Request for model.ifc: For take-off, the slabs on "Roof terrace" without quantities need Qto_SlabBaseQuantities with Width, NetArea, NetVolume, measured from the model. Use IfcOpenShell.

First a look at what the model holds.

```python
import ifcopenshell
import ifcopenshell.util.element
import ifcopenshell.util.unit

model = ifcopenshell.open("model.ifc")
print(model.schema)
for unit_type in ("LENGTHUNIT", "AREAUNIT", "VOLUMEUNIT"):
    print(unit_type, ifcopenshell.util.unit.calculate_unit_scale(model, unit_type))
storey = next(s for s in model.by_type("IfcBuildingStorey") if s.Name == "Roof terrace")
slabs = [e for e in ifcopenshell.util.element.get_decomposition(storey) if e.is_a("IfcSlab")]
for e in sorted(slabs, key=lambda e: e.id()):
    print(e.id(), e.is_a(), e.Name, list(ifcopenshell.util.element.get_psets(e, qtos_only=True)), sep=" | ")
```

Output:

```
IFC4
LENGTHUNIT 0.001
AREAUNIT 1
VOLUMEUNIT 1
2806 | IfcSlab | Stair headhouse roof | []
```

```python
import ifcopenshell
import ifcopenshell.api.pset
import ifcopenshell.geom
import ifcopenshell.util.element
import ifcopenshell.util.shape
import ifcopenshell.util.unit

model = ifcopenshell.open("model.ifc")
unit_scale = ifcopenshell.util.unit.calculate_unit_scale(model)
area_scale = ifcopenshell.util.unit.calculate_unit_scale(model, "AREAUNIT")
volume_scale = ifcopenshell.util.unit.calculate_unit_scale(model, "VOLUMEUNIT")
settings = ifcopenshell.geom.settings()

storey = next(s for s in model.by_type("IfcBuildingStorey") if s.Name == "Roof terrace")
slabs = [e for e in ifcopenshell.util.element.get_decomposition(storey) if e.is_a("IfcSlab")]

for e in sorted(slabs, key=lambda e: e.id()):
    if ifcopenshell.util.element.get_psets(e, qtos_only=True, should_inherit=False):
        continue
    # Geometry comes back in metres, in the element's own axes.
    shape = ifcopenshell.geom.create_shape(settings, e)
    values = {
        "Width": ifcopenshell.util.shape.get_z(shape.geometry) / unit_scale,
        "NetArea": ifcopenshell.util.shape.get_footprint_area(shape.geometry) / area_scale,
        "NetVolume": ifcopenshell.util.shape.get_volume(shape.geometry) / volume_scale,
    }
    qto = ifcopenshell.api.pset.add_qto(model, product=e, name="Qto_SlabBaseQuantities")
    ifcopenshell.api.pset.edit_qto(model, qto=qto, properties=values)
    print(e.id(), {k: round(v, 3) for k, v in values.items()})

model.write("model_v2.ifc")
```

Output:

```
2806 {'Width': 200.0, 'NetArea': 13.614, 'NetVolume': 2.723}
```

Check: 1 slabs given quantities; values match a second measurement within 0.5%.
